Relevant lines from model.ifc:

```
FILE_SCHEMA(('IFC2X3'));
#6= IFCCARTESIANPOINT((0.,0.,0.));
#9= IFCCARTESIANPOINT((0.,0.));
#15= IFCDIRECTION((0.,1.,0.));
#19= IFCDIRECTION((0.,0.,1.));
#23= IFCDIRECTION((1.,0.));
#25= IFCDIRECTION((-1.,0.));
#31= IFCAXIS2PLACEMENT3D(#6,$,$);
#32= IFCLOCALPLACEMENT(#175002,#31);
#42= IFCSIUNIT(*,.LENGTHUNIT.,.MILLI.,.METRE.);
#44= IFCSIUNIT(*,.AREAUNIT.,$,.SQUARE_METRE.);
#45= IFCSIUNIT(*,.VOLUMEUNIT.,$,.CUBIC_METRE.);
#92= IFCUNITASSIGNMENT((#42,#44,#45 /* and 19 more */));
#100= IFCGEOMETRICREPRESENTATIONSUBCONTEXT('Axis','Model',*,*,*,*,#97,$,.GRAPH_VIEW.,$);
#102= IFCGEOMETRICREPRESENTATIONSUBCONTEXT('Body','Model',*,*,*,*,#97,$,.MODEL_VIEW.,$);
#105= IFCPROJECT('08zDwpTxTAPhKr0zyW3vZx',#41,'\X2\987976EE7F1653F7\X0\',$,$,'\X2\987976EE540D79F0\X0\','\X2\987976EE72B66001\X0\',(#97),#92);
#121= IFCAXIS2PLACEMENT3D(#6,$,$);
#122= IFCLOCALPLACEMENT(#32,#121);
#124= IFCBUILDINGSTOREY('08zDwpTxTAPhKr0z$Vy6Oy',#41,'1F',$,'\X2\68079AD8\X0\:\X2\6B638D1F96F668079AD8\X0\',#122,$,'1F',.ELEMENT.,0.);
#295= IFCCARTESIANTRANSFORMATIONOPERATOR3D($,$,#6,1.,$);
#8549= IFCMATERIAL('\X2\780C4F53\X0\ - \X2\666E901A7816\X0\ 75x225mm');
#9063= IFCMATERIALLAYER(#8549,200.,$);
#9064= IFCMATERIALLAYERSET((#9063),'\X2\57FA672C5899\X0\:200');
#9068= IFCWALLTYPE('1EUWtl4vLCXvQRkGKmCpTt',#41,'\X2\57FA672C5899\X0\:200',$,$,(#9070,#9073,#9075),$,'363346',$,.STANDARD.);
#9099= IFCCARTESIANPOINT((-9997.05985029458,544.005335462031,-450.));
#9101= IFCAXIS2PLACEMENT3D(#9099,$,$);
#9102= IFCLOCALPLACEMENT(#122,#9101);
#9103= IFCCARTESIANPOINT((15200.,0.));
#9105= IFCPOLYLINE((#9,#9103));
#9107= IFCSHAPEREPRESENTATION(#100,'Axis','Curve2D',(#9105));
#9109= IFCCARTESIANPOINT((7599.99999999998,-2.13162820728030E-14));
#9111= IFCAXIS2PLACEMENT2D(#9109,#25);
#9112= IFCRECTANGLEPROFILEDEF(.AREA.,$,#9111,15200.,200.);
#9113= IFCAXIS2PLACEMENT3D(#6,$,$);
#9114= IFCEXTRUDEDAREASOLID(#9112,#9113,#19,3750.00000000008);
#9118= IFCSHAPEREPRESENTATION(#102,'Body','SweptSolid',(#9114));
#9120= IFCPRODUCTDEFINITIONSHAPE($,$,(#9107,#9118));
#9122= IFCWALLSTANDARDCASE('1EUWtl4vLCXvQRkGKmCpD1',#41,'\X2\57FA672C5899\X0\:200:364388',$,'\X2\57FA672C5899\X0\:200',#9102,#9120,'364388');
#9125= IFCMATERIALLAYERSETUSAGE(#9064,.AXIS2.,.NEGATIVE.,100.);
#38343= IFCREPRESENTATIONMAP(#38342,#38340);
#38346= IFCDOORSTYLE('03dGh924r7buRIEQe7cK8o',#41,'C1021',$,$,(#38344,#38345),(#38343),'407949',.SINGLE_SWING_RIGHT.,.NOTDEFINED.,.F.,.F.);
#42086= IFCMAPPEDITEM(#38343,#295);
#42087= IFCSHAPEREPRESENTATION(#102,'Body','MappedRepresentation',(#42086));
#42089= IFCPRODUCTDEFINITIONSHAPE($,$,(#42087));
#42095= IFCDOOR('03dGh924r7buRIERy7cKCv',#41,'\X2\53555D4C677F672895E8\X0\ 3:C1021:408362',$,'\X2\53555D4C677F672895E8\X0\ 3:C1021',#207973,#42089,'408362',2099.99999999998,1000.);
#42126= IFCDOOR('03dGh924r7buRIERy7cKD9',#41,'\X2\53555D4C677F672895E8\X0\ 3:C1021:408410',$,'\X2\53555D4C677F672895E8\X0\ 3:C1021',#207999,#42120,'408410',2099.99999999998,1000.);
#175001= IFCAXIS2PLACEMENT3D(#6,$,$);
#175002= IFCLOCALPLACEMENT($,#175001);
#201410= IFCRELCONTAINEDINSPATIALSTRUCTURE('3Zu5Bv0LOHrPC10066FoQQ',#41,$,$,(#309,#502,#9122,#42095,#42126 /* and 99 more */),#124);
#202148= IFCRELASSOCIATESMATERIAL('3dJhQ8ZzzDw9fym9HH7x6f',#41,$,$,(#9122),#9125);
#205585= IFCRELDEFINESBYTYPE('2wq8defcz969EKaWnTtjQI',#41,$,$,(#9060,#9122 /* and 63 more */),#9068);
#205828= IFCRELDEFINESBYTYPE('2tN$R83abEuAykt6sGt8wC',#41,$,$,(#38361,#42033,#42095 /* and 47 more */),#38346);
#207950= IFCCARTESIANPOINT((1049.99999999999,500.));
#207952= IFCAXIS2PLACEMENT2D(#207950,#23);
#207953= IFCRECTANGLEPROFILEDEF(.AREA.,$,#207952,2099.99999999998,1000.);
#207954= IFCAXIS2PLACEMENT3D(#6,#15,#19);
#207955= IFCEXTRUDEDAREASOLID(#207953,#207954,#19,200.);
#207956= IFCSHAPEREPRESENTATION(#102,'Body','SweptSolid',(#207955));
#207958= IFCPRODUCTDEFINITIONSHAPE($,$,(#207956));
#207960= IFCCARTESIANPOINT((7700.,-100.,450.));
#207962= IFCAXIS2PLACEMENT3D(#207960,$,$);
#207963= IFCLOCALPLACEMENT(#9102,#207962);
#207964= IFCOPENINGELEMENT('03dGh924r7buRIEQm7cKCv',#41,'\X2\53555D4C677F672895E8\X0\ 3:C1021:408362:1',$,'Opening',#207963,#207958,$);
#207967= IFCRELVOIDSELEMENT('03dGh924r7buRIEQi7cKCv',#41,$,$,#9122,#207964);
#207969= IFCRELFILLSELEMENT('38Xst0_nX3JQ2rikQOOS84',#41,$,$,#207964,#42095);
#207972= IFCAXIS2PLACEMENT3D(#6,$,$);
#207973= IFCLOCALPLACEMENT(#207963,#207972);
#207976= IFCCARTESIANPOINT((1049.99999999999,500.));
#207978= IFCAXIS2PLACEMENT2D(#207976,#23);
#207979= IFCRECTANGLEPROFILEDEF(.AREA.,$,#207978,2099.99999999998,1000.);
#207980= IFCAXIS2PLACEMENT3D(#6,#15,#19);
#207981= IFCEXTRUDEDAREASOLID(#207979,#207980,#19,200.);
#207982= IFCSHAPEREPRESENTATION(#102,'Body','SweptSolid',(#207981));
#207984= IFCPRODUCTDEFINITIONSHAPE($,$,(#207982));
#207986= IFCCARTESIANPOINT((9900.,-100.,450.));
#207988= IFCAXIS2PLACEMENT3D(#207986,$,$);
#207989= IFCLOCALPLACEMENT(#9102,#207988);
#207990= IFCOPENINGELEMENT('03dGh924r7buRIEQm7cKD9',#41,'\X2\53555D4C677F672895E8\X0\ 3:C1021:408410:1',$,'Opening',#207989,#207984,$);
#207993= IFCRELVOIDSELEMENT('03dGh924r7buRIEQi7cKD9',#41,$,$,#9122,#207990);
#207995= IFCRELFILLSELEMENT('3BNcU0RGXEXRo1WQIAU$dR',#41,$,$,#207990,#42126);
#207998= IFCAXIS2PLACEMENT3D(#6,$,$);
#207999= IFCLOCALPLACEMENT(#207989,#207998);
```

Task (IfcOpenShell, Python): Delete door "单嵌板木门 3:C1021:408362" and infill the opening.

```python
import ifcopenshell
import ifcopenshell.api.feature
import ifcopenshell.api.root
import ifcopenshell.geom
import ifcopenshell.util.shape

model = ifcopenshell.open("model.ifc")
settings = ifcopenshell.geom.settings()


def volume(element):
    """Net volume in cubic metres, openings subtracted."""
    shape = ifcopenshell.geom.create_shape(settings, element)
    return ifcopenshell.util.shape.get_volume(shape.geometry)


door = model.by_guid("03dGh924r7buRIERy7cKCv")
opening = door.FillsVoids[0].RelatingOpeningElement
wall = opening.VoidsElements[0].RelatingBuildingElement
before = volume(wall)

ifcopenshell.api.root.remove_product(model, product=door)
ifcopenshell.api.feature.remove_feature(model, feature=opening)

after = volume(wall)

print(f"wall volume {before:.3f} -> {after:.3f} m3")

model.write("model_updated.ifc")
```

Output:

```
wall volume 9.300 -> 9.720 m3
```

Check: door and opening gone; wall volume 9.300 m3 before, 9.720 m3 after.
